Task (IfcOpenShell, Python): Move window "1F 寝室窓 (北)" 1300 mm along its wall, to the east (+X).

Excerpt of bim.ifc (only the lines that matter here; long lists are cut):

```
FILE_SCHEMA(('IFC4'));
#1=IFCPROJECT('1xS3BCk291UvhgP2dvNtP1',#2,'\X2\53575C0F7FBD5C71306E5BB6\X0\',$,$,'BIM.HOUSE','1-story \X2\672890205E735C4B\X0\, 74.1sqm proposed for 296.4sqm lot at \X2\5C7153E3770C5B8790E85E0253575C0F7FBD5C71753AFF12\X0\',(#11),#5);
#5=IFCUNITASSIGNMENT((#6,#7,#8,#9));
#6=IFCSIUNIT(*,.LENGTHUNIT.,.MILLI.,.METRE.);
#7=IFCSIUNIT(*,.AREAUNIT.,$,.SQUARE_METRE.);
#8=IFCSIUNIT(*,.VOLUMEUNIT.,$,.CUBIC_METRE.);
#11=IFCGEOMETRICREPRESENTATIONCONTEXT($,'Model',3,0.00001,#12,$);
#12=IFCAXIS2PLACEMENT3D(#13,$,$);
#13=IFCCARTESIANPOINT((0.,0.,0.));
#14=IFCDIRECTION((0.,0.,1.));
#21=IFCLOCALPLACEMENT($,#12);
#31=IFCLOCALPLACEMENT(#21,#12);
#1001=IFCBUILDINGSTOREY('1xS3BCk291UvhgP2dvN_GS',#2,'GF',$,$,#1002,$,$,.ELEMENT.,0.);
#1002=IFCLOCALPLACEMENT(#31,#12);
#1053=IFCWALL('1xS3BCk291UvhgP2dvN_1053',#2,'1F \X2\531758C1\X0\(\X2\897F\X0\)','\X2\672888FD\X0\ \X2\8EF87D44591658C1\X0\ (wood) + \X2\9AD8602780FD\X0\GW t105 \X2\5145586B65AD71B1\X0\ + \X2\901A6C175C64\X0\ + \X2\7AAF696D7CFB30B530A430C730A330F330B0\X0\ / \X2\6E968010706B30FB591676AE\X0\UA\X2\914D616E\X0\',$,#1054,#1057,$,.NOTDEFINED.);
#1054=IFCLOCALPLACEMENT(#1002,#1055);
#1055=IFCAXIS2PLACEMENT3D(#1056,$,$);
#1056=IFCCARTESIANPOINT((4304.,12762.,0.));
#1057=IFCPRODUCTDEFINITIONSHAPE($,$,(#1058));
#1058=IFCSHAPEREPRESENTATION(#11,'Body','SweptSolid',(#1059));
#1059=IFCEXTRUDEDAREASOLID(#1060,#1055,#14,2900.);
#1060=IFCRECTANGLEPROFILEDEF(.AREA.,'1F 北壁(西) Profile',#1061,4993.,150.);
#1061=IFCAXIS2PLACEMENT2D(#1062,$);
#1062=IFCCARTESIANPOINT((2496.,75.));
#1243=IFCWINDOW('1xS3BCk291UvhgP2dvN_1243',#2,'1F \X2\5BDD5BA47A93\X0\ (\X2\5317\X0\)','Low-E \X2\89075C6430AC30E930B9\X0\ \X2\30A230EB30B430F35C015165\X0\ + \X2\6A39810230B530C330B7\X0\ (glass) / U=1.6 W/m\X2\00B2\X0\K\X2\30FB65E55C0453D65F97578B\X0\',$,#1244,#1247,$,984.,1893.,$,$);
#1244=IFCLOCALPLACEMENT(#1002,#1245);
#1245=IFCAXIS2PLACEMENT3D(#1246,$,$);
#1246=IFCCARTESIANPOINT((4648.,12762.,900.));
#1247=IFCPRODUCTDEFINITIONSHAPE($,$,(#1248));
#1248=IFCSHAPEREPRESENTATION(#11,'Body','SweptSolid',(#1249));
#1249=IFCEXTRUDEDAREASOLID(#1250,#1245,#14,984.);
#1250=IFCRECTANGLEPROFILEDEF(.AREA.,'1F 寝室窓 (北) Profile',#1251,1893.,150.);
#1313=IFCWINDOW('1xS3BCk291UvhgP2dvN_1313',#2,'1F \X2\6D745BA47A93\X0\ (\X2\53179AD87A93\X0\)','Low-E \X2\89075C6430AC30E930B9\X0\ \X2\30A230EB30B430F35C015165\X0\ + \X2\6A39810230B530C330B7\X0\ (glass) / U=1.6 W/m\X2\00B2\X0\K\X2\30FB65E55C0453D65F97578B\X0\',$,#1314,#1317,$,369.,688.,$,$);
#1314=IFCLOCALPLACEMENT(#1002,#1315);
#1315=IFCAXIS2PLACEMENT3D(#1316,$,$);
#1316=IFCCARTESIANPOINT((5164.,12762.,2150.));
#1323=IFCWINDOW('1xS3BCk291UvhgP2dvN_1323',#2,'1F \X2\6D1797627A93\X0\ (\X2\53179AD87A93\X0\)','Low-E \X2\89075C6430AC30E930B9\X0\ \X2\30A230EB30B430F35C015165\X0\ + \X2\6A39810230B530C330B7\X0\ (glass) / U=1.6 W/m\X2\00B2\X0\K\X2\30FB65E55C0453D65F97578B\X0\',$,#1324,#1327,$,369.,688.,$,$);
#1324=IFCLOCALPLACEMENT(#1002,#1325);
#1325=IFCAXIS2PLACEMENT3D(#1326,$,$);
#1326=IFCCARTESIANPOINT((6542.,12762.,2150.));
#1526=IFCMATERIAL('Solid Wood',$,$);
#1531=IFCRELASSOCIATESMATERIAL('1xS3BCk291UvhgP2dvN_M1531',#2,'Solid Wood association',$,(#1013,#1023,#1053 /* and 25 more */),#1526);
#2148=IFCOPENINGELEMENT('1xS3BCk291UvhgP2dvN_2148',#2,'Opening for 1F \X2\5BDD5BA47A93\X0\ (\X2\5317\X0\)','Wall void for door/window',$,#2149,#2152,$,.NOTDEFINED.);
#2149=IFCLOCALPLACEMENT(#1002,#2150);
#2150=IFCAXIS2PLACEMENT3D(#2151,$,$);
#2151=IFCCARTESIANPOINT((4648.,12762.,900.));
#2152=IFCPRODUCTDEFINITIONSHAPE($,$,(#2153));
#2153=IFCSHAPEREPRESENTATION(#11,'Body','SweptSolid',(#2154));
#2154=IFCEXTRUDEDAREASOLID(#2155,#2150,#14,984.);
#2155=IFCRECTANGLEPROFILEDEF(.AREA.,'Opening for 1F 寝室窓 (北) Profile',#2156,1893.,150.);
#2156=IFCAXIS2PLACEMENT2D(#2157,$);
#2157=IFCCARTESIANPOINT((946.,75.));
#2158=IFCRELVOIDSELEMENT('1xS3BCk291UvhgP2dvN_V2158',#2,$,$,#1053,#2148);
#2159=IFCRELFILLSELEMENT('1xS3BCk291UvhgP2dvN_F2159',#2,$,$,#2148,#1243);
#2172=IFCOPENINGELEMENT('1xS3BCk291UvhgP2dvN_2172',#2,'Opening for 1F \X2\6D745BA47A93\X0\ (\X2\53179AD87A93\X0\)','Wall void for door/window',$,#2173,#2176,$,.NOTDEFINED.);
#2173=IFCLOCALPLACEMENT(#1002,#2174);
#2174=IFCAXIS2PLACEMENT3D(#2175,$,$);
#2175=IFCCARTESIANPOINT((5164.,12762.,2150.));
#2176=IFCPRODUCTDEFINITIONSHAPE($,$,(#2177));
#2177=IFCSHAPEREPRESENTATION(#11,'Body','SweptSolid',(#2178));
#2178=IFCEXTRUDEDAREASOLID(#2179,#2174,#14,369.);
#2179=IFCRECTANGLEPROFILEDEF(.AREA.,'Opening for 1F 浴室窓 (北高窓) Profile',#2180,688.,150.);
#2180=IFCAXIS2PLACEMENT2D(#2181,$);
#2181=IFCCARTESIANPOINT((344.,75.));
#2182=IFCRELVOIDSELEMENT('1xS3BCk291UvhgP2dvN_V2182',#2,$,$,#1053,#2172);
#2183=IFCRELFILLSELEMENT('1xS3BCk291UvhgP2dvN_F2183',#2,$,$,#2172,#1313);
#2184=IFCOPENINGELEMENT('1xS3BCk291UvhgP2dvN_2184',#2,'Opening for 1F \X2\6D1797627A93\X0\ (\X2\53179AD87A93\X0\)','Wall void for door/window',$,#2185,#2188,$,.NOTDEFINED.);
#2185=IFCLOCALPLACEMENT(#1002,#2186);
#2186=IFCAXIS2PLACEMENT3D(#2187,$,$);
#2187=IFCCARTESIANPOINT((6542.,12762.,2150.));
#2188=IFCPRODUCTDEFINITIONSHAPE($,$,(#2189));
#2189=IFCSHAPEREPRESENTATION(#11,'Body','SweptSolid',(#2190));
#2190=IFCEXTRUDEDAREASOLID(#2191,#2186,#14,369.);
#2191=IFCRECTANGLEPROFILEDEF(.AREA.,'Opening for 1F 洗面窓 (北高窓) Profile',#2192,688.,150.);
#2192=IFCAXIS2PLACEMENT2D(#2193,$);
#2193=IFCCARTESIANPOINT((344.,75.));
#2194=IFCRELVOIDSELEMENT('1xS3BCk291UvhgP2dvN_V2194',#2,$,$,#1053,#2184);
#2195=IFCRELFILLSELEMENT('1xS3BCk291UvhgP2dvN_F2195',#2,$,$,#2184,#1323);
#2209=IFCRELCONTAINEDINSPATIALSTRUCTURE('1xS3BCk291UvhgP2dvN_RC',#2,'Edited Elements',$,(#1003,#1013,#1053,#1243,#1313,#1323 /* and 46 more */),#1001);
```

```python
import ifcopenshell
import ifcopenshell.api.geometry
import ifcopenshell.util.placement
import ifcopenshell.util.unit

model = ifcopenshell.open("bim.ifc")
unit_scale = ifcopenshell.util.unit.calculate_unit_scale(model)

window = model.by_id(1243)
opening = window.FillsVoids[0].RelatingOpeningElement
wall = opening.VoidsElements[0].RelatingBuildingElement

wall_matrix = ifcopenshell.util.placement.get_local_placement(wall.ObjectPlacement)
shift = wall_matrix[:3, 0] * 1.3 / unit_scale
before = ifcopenshell.util.placement.get_local_placement(window.ObjectPlacement)[:3, 3].copy()

# The window is not placed relative to its opening, so move both.
for product in (opening, window):
    matrix = ifcopenshell.util.placement.get_local_placement(product.ObjectPlacement)
    matrix[:3, 3] += shift
    ifcopenshell.api.geometry.edit_object_placement(model, product=product, matrix=matrix, is_si=False)

after = ifcopenshell.util.placement.get_local_placement(window.ObjectPlacement)[:3, 3]
print("window moved by", (after - before).round(3) + 0.0)

model.write("bim_edited.ifc")
```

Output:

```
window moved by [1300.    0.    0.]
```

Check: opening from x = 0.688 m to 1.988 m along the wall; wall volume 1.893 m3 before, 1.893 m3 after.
